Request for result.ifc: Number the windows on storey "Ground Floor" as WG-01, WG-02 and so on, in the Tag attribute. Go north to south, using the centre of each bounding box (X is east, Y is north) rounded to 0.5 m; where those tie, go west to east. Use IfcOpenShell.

First a look at what the model holds.

```python
import ifcopenshell
import ifcopenshell.util.element
import ifcopenshell.util.placement

model = ifcopenshell.open("result.ifc")
print(model.schema)
storey = next(s for s in model.by_type("IfcBuildingStorey") if s.Name == "Ground Floor")
windows = [e for e in ifcopenshell.util.element.get_decomposition(storey) if e.is_a("IfcWindow")]
for e in sorted(windows, key=lambda e: e.id()):
    origin = ifcopenshell.util.placement.get_local_placement(e.ObjectPlacement)[:3, 3]
    print(e.id(), e.Tag, e.Name, origin.round(2) + 0.0, sep=" | ")
```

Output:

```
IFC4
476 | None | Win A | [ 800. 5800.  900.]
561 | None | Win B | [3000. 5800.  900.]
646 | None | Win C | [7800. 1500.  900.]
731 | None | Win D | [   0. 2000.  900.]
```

```python
import ifcopenshell
import ifcopenshell.geom
import ifcopenshell.util.element
import ifcopenshell.util.shape

model = ifcopenshell.open("result.ifc")
settings = ifcopenshell.geom.settings()
settings.set("use-world-coords", True)


def centre(element):
    shape = ifcopenshell.geom.create_shape(settings, element)
    return ifcopenshell.util.shape.get_bbox_centroid(shape.geometry)


storey = next(s for s in model.by_type("IfcBuildingStorey") if s.Name == "Ground Floor")
windows = [e for e in ifcopenshell.util.element.get_decomposition(storey) if e.is_a("IfcWindow")]

# Insertion points can sit at a corner or the storey origin, so sort by the geometry (in metres).
centres = {e: centre(e) for e in windows}
windows.sort(key=lambda e: (-round(centres[e][1] / 0.5), centres[e][0]))

for i, e in enumerate(windows, start=1):
    number = f"WG-{i:02d}"
    e.Tag = number
    print(e.id(), number)

model.write("result_v2.ifc")
```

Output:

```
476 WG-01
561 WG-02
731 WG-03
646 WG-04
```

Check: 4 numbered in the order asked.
